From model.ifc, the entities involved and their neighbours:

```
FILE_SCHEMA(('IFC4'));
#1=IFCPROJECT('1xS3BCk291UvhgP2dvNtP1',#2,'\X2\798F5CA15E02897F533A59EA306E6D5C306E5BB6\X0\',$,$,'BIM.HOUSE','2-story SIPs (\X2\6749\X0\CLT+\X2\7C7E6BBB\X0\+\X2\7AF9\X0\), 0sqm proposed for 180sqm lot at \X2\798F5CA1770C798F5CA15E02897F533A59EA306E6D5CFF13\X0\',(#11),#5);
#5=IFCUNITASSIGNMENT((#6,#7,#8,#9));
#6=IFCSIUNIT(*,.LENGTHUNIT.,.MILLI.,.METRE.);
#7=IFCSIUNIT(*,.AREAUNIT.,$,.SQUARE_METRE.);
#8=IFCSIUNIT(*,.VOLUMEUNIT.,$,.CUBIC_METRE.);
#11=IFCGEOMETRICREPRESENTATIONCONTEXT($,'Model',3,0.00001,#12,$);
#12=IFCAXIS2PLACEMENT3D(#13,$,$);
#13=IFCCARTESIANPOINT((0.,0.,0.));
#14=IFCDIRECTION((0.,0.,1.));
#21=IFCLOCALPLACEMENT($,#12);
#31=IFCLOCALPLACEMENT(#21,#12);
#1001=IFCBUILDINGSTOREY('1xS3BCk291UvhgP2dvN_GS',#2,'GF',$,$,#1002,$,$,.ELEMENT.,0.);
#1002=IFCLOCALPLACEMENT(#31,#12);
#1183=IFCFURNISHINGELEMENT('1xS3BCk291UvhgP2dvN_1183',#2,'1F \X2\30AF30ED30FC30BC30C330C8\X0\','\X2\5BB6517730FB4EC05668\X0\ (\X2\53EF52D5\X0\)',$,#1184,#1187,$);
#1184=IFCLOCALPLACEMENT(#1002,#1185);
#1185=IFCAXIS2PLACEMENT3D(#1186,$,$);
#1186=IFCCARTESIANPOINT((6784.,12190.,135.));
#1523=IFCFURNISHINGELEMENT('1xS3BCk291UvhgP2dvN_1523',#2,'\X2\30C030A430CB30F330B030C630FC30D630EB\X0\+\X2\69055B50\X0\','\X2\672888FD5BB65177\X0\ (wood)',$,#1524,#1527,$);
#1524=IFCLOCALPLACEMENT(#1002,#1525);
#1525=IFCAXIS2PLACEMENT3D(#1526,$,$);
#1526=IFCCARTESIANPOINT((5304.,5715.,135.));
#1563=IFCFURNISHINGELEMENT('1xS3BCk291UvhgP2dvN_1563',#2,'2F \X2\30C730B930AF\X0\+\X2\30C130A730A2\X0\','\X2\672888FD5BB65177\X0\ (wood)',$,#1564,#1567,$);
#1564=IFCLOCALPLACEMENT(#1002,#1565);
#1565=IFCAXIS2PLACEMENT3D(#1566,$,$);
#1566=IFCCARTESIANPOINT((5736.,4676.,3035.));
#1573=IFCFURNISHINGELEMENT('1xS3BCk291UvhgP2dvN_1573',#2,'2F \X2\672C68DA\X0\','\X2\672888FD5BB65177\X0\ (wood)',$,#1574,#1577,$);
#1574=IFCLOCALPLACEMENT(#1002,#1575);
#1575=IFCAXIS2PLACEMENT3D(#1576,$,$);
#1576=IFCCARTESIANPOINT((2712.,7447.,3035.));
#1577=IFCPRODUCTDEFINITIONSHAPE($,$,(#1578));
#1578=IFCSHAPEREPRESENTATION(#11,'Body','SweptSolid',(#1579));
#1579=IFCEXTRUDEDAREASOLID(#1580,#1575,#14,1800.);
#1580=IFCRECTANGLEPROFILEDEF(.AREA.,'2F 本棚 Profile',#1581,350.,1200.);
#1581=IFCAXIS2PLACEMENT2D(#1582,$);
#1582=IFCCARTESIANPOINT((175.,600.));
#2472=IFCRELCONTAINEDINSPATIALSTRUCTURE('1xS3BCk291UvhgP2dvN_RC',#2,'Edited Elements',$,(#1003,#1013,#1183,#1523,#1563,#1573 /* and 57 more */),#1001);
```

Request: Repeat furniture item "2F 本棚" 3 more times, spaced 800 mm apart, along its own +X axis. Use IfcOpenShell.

```python
import ifcopenshell
import ifcopenshell.api.geometry
import ifcopenshell.api.root
import ifcopenshell.util.element
import ifcopenshell.util.placement

model = ifcopenshell.open("model.ifc")


def reuse_history(source, copy):
    """copy_class also copies each property set's owner history, people and application; keep the originals."""
    for rel in copy.IsDefinedBy:
        if rel.is_a("IfcRelDefinesByProperties") and (history := rel.RelatingPropertyDefinition.OwnerHistory):
            rel.RelatingPropertyDefinition.OwnerHistory = source.OwnerHistory
            ifcopenshell.util.element.remove_deep2(model, history)


source = model.by_guid("1xS3BCk291UvhgP2dvN_1573")
base = ifcopenshell.util.placement.get_local_placement(source.ObjectPlacement)
step = base[:3, 0] * 800.0

for i in range(1, 4):
    copy = ifcopenshell.api.root.copy_class(model, product=source)
    copy.Representation = ifcopenshell.util.element.copy_deep(
        model, source.Representation, exclude=["IfcGeometricRepresentationContext", "IfcRepresentationMap"]
    )
    reuse_history(source, copy)
    matrix = base.copy()
    matrix[:3, 3] += i * step
    print("added at", matrix[:3, 3].round(3) + 0.0)
    ifcopenshell.api.geometry.edit_object_placement(model, product=copy, matrix=matrix, is_si=False)

model.write("model_v2.ifc")
```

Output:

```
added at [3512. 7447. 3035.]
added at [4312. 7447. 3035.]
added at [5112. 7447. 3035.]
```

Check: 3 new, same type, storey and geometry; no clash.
